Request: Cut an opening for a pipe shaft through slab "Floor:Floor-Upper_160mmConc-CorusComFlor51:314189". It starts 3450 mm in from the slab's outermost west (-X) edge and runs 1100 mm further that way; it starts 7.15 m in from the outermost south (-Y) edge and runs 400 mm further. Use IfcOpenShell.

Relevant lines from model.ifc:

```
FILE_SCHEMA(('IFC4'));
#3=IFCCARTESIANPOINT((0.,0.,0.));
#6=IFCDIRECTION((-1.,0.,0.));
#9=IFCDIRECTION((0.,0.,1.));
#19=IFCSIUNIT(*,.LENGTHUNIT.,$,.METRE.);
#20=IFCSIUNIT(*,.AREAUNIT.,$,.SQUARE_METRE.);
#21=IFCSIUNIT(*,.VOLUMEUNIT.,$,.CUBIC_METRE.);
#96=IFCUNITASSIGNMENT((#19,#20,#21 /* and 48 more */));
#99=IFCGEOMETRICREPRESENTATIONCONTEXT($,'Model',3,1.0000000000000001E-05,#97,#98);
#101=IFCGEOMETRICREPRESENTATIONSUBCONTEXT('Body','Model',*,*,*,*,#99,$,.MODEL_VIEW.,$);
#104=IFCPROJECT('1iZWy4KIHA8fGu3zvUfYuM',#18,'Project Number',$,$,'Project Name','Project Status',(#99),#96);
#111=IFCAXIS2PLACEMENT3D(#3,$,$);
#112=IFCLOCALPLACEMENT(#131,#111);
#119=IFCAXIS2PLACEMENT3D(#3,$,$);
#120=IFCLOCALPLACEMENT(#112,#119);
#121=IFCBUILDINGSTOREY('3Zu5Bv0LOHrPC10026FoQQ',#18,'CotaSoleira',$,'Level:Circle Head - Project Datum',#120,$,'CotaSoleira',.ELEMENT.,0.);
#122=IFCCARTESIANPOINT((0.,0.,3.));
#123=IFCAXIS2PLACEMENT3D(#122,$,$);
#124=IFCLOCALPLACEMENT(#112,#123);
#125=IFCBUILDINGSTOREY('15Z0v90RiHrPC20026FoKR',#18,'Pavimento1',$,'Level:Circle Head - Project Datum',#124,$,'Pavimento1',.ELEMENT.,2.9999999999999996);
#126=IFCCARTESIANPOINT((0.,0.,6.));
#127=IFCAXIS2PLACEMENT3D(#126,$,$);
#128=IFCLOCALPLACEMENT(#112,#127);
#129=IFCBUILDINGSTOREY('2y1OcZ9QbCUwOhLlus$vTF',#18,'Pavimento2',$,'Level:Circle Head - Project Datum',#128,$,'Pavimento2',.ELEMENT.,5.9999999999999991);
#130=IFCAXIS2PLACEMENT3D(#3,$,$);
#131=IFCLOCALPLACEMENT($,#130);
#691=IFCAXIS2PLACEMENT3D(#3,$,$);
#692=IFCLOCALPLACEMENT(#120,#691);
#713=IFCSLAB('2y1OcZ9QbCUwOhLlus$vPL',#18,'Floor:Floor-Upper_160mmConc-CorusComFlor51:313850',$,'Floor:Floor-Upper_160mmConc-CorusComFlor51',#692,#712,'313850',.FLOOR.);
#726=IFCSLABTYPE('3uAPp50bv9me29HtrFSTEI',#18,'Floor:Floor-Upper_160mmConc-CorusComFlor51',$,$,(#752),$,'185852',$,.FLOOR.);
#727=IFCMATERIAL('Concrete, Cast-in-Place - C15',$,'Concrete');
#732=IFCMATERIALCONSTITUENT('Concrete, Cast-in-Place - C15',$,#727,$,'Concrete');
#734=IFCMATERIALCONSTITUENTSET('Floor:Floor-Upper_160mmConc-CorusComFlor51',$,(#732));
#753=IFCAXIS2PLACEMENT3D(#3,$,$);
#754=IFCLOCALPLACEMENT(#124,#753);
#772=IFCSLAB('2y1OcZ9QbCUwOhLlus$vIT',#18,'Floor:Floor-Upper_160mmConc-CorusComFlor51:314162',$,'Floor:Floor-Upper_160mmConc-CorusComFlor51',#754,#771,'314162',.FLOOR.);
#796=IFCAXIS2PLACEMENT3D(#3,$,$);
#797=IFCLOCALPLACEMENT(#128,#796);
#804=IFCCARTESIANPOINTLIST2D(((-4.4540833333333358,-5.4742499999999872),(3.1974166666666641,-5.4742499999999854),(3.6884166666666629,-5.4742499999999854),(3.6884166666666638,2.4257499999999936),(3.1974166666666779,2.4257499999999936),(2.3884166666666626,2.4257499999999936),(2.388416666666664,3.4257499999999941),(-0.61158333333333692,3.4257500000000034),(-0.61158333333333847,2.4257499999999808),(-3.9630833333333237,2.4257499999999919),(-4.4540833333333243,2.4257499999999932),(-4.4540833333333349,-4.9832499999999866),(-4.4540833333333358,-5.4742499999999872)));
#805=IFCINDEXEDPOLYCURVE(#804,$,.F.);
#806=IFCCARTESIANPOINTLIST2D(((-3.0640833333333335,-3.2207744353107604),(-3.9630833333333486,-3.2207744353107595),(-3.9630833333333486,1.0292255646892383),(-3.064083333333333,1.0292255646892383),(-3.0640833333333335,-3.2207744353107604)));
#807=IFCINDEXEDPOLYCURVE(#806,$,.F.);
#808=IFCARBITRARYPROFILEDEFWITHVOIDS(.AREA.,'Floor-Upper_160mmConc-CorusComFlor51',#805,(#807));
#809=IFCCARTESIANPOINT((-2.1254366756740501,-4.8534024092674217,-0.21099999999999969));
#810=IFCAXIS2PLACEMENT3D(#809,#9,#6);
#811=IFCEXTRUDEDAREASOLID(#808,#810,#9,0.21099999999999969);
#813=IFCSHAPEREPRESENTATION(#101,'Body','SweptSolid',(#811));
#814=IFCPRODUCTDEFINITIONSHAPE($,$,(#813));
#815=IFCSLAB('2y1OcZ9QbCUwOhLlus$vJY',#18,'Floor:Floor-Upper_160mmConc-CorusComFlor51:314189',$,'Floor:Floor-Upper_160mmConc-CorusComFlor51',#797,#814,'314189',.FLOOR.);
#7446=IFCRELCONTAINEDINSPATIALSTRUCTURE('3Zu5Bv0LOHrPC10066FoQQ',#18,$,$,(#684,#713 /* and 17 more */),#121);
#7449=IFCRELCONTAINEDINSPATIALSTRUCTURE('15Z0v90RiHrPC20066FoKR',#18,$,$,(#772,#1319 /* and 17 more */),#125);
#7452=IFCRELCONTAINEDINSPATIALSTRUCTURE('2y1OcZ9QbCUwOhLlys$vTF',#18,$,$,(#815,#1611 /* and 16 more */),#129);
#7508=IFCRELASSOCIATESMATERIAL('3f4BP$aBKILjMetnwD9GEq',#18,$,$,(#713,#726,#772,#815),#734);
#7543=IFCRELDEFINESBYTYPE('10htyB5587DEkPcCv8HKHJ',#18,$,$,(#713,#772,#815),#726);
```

```python
import numpy as np
import ifcopenshell
import ifcopenshell.api.feature
import ifcopenshell.api.geometry
import ifcopenshell.api.root
import ifcopenshell.geom
import ifcopenshell.util.placement
import ifcopenshell.util.representation
import ifcopenshell.util.shape
import ifcopenshell.util.unit

model = ifcopenshell.open("model.ifc")
unit_scale = ifcopenshell.util.unit.calculate_unit_scale(model)
settings = ifcopenshell.geom.settings()


def volume(element):
    """Net volume in cubic metres, openings subtracted."""
    shape = ifcopenshell.geom.create_shape(settings, element)
    return ifcopenshell.util.shape.get_volume(shape.geometry)


slab = model.by_guid("2y1OcZ9QbCUwOhLlus$vJY")
before = volume(slab)

# Extent in the slab's own axes, in metres. The edges named are its -X and -Y sides.
slab_shape = ifcopenshell.geom.create_shape(settings, slab)
vertices = ifcopenshell.util.shape.get_vertices(slab_shape.geometry)
x_min, y_min, bottom = vertices.min(axis=0)
top = vertices[:, 2].max()

opening = ifcopenshell.api.root.create_entity(model, ifc_class="IfcOpeningElement", name="Pipe shaft opening", predefined_type="OPENING")
context = ifcopenshell.util.representation.get_context(model, "Model", "Body", "MODEL_VIEW")
width, depth = 1.1, 0.4
outline = [(0.0, 0.0), (width, 0.0), (width, depth), (0.0, depth), (0.0, 0.0)]
# Overshoot both faces by 50 mm so the cut is clean.
shape = ifcopenshell.api.geometry.add_slab_representation(
    model, context=context, depth=top - bottom + 0.1, polyline=outline
)
ifcopenshell.api.geometry.assign_representation(model, product=opening, representation=shape)

matrix = ifcopenshell.util.placement.get_local_placement(slab.ObjectPlacement)
matrix[:, 3] = matrix @ np.append(np.array([x_min + 3.45, y_min + 7.15, bottom - 0.05]) / unit_scale, 1.0)
ifcopenshell.api.geometry.edit_object_placement(model, product=opening, matrix=matrix, is_si=False)
ifcopenshell.api.feature.add_feature(model, feature=opening, element=slab)

after = volume(slab)

print(f"slab volume {before:.3f} -> {after:.3f} m3")

model.write("model_edited.ifc")
```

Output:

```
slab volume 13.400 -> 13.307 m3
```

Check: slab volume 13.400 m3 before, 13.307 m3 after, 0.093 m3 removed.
